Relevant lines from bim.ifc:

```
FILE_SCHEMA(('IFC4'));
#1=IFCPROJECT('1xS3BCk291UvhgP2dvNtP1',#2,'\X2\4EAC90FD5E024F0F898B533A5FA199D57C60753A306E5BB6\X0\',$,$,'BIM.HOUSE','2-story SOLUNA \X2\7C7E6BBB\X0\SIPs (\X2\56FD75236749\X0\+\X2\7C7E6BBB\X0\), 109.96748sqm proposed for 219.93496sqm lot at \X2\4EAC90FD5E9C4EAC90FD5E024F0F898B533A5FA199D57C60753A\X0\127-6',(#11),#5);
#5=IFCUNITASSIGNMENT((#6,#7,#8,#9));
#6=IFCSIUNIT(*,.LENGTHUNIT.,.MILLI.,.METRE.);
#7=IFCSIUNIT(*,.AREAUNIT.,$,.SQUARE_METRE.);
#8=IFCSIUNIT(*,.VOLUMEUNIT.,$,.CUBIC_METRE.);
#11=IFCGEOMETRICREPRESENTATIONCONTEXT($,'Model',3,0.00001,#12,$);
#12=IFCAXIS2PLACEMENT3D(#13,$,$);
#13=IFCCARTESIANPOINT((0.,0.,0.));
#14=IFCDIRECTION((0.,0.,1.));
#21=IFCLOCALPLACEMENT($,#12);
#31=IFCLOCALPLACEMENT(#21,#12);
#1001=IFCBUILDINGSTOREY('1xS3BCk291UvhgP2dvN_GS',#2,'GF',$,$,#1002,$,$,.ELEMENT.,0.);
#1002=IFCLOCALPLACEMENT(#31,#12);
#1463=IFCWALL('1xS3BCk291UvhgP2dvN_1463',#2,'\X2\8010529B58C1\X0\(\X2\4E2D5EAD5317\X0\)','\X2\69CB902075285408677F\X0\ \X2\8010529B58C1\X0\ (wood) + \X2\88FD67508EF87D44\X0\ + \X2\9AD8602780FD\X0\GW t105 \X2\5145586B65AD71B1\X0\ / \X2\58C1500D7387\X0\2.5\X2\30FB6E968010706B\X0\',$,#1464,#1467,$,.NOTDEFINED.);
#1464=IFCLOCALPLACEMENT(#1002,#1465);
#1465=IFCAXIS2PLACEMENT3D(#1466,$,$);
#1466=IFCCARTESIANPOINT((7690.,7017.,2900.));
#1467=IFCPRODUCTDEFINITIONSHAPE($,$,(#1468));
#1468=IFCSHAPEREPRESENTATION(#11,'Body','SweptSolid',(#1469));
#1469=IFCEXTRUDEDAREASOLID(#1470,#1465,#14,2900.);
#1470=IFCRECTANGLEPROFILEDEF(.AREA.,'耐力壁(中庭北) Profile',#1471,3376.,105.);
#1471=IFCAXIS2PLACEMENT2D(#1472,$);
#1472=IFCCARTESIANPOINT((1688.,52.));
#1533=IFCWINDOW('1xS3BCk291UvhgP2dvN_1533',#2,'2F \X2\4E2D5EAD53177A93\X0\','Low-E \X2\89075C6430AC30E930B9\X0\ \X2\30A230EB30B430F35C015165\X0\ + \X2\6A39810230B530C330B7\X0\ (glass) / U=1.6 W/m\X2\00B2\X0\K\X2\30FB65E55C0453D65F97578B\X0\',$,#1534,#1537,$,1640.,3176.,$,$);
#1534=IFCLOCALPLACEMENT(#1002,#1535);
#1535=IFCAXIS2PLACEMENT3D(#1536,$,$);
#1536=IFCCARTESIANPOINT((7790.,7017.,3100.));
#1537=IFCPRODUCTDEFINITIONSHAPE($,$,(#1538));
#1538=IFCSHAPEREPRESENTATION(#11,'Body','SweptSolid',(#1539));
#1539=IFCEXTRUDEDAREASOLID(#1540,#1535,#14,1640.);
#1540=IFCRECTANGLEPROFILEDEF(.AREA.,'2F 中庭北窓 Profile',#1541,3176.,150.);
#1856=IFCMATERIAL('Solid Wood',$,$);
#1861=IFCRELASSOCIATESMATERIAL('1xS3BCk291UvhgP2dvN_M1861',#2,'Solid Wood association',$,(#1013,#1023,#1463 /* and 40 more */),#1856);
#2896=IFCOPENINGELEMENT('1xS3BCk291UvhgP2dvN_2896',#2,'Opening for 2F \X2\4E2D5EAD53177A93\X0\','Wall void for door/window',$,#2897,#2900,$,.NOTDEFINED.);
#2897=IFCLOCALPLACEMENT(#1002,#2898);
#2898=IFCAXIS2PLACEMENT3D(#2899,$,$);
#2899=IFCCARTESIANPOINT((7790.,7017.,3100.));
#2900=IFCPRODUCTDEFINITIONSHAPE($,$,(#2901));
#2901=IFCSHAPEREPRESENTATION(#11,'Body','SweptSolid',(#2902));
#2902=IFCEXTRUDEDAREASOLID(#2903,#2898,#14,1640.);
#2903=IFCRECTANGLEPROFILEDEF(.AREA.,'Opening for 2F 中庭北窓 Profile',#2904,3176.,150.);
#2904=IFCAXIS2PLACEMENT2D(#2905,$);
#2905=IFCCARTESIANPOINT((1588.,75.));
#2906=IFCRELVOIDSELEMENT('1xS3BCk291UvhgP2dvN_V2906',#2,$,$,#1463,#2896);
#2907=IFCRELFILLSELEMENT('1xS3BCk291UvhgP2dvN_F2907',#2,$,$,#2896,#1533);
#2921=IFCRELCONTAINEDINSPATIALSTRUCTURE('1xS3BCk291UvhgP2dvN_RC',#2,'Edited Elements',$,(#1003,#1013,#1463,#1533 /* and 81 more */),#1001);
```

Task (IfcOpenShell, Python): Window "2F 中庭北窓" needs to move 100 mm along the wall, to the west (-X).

```python
import ifcopenshell
import ifcopenshell.api.geometry
import ifcopenshell.util.placement
import ifcopenshell.util.unit

model = ifcopenshell.open("bim.ifc")
unit_scale = ifcopenshell.util.unit.calculate_unit_scale(model)

window = model.by_guid("1xS3BCk291UvhgP2dvN_1533")
opening = window.FillsVoids[0].RelatingOpeningElement
wall = opening.VoidsElements[0].RelatingBuildingElement

wall_matrix = ifcopenshell.util.placement.get_local_placement(wall.ObjectPlacement)
shift = wall_matrix[:3, 0] * -0.1 / unit_scale
before = ifcopenshell.util.placement.get_local_placement(window.ObjectPlacement)[:3, 3].copy()

# The window is not placed relative to its opening, so move both.
for product in (opening, window):
    matrix = ifcopenshell.util.placement.get_local_placement(product.ObjectPlacement)
    matrix[:3, 3] += shift
    ifcopenshell.api.geometry.edit_object_placement(model, product=product, matrix=matrix, is_si=False)

after = ifcopenshell.util.placement.get_local_placement(window.ObjectPlacement)[:3, 3]
print("window moved by", (after - before).round(3) + 0.0)

model.write("bim_rev.ifc")
```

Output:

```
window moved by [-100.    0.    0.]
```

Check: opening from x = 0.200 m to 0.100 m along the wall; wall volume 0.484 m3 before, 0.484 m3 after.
